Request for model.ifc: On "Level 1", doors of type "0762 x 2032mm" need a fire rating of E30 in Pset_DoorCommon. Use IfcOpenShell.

First a look at what the model holds.

```python
import ifcopenshell
import ifcopenshell.util.element

model = ifcopenshell.open("model.ifc")
print(model.schema)
storey = next(s for s in model.by_type("IfcBuildingStorey") if s.Name == "Level 1")
doors = [e for e in ifcopenshell.util.element.get_decomposition(storey) if e.is_a("IfcDoor")]
seen = {}
for e in doors:
    element_type = ifcopenshell.util.element.get_type(e)
    key = (element_type.Name if element_type != e and element_type else None, ifcopenshell.util.element.get_pset(e, "Pset_DoorCommon", "FireRating"))
    seen[key] = seen.get(key, 0) + 1
for (name, value), count in sorted(seen.items(), key=str):
    print(count, "x", name, "|", value)
```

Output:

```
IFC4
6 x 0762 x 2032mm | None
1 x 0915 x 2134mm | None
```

```python
import ifcopenshell
import ifcopenshell.api.pset
import ifcopenshell.util.element

model = ifcopenshell.open("model.ifc")

storey = next(s for s in model.by_type("IfcBuildingStorey") if s.Name == "Level 1")
doors = [e for e in ifcopenshell.util.element.get_decomposition(storey) if e.is_a("IfcDoor")]

count = 0
for e in doors:
    element_type = ifcopenshell.util.element.get_type(e)
    if element_type in (None, e) or element_type.Name != "0762 x 2032mm":
        continue
    # add_pset returns the element's existing set when there is one.
    pset = ifcopenshell.api.pset.add_pset(model, product=e, name="Pset_DoorCommon")
    ifcopenshell.api.pset.edit_pset(model, pset=pset, properties={"FireRating": "E30"})
    count += 1

print(count, "doors updated")

model.write("model_v2.ifc")
```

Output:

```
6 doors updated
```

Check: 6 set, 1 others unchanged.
